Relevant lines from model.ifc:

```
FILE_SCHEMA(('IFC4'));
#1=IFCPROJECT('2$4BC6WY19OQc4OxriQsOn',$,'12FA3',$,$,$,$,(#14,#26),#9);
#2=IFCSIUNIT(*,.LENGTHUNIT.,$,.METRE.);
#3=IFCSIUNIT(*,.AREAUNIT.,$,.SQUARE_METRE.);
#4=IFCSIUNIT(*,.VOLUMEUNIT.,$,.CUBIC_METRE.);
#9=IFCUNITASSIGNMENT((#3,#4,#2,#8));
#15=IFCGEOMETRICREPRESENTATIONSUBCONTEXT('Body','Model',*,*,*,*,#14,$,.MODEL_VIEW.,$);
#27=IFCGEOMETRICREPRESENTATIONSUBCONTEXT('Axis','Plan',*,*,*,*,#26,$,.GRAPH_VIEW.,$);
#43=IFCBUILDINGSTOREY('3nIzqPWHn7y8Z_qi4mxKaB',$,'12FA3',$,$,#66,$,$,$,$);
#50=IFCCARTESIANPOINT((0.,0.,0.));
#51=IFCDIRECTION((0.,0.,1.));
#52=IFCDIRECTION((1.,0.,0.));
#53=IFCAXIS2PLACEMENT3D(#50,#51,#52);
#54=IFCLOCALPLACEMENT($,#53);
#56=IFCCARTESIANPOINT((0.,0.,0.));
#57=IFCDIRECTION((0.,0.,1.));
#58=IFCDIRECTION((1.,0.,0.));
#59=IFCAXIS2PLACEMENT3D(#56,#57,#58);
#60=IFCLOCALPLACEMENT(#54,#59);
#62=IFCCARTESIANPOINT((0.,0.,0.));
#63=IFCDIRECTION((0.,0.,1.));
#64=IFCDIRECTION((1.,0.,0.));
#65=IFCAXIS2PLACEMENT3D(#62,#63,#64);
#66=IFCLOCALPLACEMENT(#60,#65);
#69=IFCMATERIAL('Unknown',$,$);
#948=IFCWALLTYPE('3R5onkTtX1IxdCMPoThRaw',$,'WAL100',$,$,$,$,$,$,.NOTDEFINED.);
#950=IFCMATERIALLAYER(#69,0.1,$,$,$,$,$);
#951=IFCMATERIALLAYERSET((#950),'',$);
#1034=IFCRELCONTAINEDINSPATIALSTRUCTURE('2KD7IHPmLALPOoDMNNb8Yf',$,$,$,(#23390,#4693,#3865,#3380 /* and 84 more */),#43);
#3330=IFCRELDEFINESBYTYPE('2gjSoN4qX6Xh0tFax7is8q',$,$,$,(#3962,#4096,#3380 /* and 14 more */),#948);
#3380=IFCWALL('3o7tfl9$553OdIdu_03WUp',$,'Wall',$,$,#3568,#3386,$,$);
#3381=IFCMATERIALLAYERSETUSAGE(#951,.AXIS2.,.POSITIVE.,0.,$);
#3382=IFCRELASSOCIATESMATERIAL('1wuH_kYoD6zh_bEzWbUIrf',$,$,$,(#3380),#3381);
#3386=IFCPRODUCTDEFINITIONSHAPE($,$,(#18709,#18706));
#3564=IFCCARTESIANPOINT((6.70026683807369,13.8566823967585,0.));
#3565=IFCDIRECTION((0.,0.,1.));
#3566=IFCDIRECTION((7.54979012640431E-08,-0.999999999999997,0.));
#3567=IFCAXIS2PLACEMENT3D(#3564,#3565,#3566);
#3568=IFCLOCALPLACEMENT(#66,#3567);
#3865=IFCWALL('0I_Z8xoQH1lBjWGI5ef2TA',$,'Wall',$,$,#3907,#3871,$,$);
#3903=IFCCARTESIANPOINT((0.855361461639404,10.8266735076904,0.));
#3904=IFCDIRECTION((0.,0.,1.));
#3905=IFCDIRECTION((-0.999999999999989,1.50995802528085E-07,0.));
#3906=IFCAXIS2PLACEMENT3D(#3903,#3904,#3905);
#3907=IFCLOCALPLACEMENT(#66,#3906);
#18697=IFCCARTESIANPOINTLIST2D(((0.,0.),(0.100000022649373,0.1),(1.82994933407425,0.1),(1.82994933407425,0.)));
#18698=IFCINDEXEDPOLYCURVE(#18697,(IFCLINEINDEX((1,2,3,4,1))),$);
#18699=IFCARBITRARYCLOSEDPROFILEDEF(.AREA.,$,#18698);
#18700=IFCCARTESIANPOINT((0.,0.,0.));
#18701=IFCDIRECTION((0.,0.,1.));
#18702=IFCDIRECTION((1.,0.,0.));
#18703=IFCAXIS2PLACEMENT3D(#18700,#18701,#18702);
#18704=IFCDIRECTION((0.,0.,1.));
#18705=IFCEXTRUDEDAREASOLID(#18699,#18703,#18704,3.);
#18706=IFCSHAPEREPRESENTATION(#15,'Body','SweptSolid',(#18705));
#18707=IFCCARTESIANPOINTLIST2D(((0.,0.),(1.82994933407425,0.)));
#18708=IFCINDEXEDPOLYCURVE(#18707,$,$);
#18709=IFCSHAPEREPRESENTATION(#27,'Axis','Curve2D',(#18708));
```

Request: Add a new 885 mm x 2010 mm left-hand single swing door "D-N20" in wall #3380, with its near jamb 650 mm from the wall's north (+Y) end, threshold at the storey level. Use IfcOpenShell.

```python
import numpy as np
import ifcopenshell
import ifcopenshell.api.feature
import ifcopenshell.api.geometry
import ifcopenshell.api.root
import ifcopenshell.api.spatial
import ifcopenshell.geom
import ifcopenshell.util.element
import ifcopenshell.util.placement
import ifcopenshell.util.representation
import ifcopenshell.util.shape
import ifcopenshell.util.unit

model = ifcopenshell.open("model.ifc")
unit_scale = ifcopenshell.util.unit.calculate_unit_scale(model)
settings = ifcopenshell.geom.settings()


def volume(element):
    """Net volume in cubic metres, openings subtracted."""
    shape = ifcopenshell.geom.create_shape(settings, element)
    return ifcopenshell.util.shape.get_volume(shape.geometry)


wall = model.by_id(3380)
storey = ifcopenshell.util.element.get_container(wall, ifc_class="IfcBuildingStorey")
context = ifcopenshell.util.representation.get_context(model, "Model", "Body", "MODEL_VIEW")
before = volume(wall)

width, height, from_end, sill = 0.885, 2.01, 0.65, 0.0  # metres

# The wall runs along its own X axis, and the end named is its -X end.
wall_shape = ifcopenshell.geom.create_shape(settings, wall)
x, y, z = ifcopenshell.util.shape.get_vertices(wall_shape.geometry).T
start = x.min() + from_end
face, thickness = float(y.min()), float(y.max() - y.min())
wall_matrix = ifcopenshell.util.placement.get_local_placement(wall.ObjectPlacement)
level = ifcopenshell.util.placement.get_local_placement(storey.ObjectPlacement)[2, 3]


def in_wall(x, y):
    """Placement at x, y metres in the wall's axes, at sill height."""
    matrix = wall_matrix.copy()
    matrix[:, 3] = wall_matrix @ np.array([x / unit_scale, y / unit_scale, 0.0, 1.0])
    matrix[2, 3] = level + sill / unit_scale
    return matrix


# Opening: a box that overshoots both wall faces by 50 mm.
opening = ifcopenshell.api.root.create_entity(model, ifc_class="IfcOpeningElement", predefined_type="OPENING")
box = ifcopenshell.api.geometry.add_wall_representation(
    model, context=context, length=width, height=height, thickness=thickness + 0.1
)
ifcopenshell.api.geometry.assign_representation(model, product=opening, representation=box)
ifcopenshell.api.geometry.edit_object_placement(model, product=opening, matrix=in_wall(start, face - 0.05), is_si=False)
ifcopenshell.api.feature.add_feature(model, feature=opening, element=wall)

door = ifcopenshell.api.root.create_entity(model, ifc_class="IfcDoor", name="D-N20", predefined_type="DOOR")
door.OverallWidth, door.OverallHeight = width / unit_scale, height / unit_scale
door.OperationType = "SINGLE_SWING_LEFT"
body = ifcopenshell.api.geometry.add_door_representation(
    model,
    context=context,
    overall_width=door.OverallWidth,
    overall_height=door.OverallHeight,
    operation_type="SINGLE_SWING_LEFT",
    lining_properties={"LiningDepth": thickness / unit_scale, "ThresholdDepth": thickness / unit_scale},
)
ifcopenshell.api.geometry.assign_representation(model, product=door, representation=body)
ifcopenshell.api.spatial.assign_container(model, products=[door], relating_structure=storey)
ifcopenshell.api.feature.add_filling(model, opening=opening, element=door)

# The lining spans the wall, so the door starts at the wall face.
ifcopenshell.api.geometry.edit_object_placement(model, product=door, matrix=in_wall(start, face), is_si=False)

after = volume(wall)

print(f"wall volume {before:.3f} -> {after:.3f} m3")

model.write("model_updated.ifc")
```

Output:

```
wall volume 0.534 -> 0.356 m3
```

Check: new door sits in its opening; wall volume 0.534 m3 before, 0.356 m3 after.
